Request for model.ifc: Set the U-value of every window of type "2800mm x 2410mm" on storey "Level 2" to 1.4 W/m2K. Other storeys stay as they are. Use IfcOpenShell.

First a look at what the model holds.

```python
import ifcopenshell
import ifcopenshell.util.element

model = ifcopenshell.open("model.ifc")
print(model.schema)
storey = next(s for s in model.by_type("IfcBuildingStorey") if s.Name == "Level 2")
windows = [e for e in ifcopenshell.util.element.get_decomposition(storey) if e.is_a("IfcWindow")]
seen = {}
for e in windows:
    element_type = ifcopenshell.util.element.get_type(e)
    key = (element_type.Name if element_type != e and element_type else None, ifcopenshell.util.element.get_pset(e, "Pset_WindowCommon", "ThermalTransmittance"))
    seen[key] = seen.get(key, 0) + 1
for (name, value), count in sorted(seen.items(), key=str):
    print(count, "x", name, "|", value)
```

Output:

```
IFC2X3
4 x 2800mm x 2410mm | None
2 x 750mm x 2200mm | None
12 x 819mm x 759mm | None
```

```python
import ifcopenshell
import ifcopenshell.api.pset
import ifcopenshell.util.element

model = ifcopenshell.open("model.ifc")

storey = next(s for s in model.by_type("IfcBuildingStorey") if s.Name == "Level 2")
windows = [e for e in ifcopenshell.util.element.get_decomposition(storey) if e.is_a("IfcWindow")]

count = 0
for e in windows:
    element_type = ifcopenshell.util.element.get_type(e)
    if element_type in (None, e) or element_type.Name != "2800mm x 2410mm":
        continue
    # add_pset returns the element's existing set when there is one.
    pset = ifcopenshell.api.pset.add_pset(model, product=e, name="Pset_WindowCommon")
    ifcopenshell.api.pset.edit_pset(model, pset=pset, properties={"ThermalTransmittance": 1.4})
    count += 1

print(count, "windows updated")

model.write("model_v2.ifc")
```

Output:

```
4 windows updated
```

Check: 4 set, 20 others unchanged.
